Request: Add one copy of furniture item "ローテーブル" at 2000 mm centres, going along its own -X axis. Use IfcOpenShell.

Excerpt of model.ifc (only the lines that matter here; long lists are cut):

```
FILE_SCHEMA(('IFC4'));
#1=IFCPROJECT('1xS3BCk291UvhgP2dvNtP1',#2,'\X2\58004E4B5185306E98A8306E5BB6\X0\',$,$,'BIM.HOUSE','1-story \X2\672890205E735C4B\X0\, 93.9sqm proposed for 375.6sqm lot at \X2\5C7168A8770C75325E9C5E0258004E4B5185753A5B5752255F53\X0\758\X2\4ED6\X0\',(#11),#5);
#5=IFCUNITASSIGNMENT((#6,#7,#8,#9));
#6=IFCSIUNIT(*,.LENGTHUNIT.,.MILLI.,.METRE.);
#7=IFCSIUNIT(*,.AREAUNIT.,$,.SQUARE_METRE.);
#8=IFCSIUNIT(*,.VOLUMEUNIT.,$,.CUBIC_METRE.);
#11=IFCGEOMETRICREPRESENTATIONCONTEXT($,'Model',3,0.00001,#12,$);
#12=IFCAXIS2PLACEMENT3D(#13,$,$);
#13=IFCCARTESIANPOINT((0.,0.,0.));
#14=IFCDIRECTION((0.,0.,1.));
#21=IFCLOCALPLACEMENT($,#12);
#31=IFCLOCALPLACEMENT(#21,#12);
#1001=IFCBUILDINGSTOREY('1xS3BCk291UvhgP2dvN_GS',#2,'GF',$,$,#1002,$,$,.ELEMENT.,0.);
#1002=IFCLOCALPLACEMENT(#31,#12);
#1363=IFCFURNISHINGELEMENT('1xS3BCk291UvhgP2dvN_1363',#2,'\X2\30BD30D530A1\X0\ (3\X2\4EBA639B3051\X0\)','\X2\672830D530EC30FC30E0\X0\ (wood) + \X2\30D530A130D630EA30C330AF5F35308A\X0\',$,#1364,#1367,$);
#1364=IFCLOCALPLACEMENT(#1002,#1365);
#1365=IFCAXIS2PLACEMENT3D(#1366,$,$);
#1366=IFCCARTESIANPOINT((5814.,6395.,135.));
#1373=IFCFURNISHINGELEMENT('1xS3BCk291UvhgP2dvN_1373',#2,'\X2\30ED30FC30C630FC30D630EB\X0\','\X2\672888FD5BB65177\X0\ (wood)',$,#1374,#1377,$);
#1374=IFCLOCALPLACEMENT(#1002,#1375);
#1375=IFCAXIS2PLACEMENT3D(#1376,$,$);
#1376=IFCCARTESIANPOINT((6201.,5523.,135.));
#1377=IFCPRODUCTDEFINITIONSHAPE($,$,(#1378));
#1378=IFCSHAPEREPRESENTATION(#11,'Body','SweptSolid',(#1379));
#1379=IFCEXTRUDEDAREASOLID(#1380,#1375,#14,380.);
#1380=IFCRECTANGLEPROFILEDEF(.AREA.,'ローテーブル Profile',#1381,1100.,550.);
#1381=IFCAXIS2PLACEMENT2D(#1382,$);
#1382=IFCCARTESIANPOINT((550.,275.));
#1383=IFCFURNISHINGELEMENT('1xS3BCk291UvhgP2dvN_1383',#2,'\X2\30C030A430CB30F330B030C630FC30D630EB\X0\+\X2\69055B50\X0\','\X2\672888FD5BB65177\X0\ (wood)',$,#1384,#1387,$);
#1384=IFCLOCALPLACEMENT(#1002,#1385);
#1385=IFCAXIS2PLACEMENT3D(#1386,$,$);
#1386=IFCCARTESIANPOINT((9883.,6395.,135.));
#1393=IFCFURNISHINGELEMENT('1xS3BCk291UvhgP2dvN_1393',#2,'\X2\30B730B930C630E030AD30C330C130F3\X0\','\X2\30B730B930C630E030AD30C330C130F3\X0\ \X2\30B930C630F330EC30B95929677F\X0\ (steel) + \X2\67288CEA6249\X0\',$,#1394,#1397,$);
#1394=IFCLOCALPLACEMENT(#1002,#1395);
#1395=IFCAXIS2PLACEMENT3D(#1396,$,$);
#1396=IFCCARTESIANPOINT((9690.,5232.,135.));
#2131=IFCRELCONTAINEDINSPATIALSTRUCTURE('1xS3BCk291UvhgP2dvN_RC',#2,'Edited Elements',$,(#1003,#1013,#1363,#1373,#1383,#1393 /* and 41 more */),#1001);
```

```python
import ifcopenshell
import ifcopenshell.api.geometry
import ifcopenshell.api.root
import ifcopenshell.util.element
import ifcopenshell.util.placement
import ifcopenshell.util.unit

model = ifcopenshell.open("model.ifc")
unit_scale = ifcopenshell.util.unit.calculate_unit_scale(model)


def reuse_history(source, copy):
    """copy_class also copies each property set's owner history, people and application; keep the originals."""
    for rel in copy.IsDefinedBy:
        if rel.is_a("IfcRelDefinesByProperties") and (history := rel.RelatingPropertyDefinition.OwnerHistory):
            rel.RelatingPropertyDefinition.OwnerHistory = source.OwnerHistory
            ifcopenshell.util.element.remove_deep2(model, history)


source = model.by_id(1373)
base = ifcopenshell.util.placement.get_local_placement(source.ObjectPlacement)
step = -base[:3, 0] * 2 / unit_scale

for i in range(1, 2):
    copy = ifcopenshell.api.root.copy_class(model, product=source)
    copy.Representation = ifcopenshell.util.element.copy_deep(
        model, source.Representation, exclude=["IfcGeometricRepresentationContext", "IfcRepresentationMap"]
    )
    reuse_history(source, copy)
    matrix = base.copy()
    matrix[:3, 3] += i * step
    print("added at", matrix[:3, 3].round(3) + 0.0)
    ifcopenshell.api.geometry.edit_object_placement(model, product=copy, matrix=matrix, is_si=False)

model.write("model_updated.ifc")
```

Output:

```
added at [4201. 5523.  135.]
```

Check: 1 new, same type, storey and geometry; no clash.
